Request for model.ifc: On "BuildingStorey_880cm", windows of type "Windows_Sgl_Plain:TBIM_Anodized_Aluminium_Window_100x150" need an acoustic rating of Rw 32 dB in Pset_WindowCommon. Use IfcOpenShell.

First a look at what the model holds.

```python
import ifcopenshell
import ifcopenshell.util.element

model = ifcopenshell.open("model.ifc")
print(model.schema)
storey = next(s for s in model.by_type("IfcBuildingStorey") if s.Name == "BuildingStorey_880cm")
windows = [e for e in ifcopenshell.util.element.get_decomposition(storey) if e.is_a("IfcWindow")]
seen = {}
for e in windows:
    element_type = ifcopenshell.util.element.get_type(e)
    key = (element_type.Name if element_type != e and element_type else None, ifcopenshell.util.element.get_pset(e, "Pset_WindowCommon", "AcousticRating"))
    seen[key] = seen.get(key, 0) + 1
for (name, value), count in sorted(seen.items(), key=str):
    print(count, "x", name, "|", value)
```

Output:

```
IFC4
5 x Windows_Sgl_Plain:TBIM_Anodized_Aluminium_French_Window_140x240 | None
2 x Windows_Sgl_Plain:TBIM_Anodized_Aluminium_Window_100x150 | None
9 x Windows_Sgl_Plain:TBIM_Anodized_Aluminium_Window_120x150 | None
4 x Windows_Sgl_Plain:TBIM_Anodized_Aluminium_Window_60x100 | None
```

```python
import ifcopenshell
import ifcopenshell.api.pset
import ifcopenshell.util.element

model = ifcopenshell.open("model.ifc")

storey = next(s for s in model.by_type("IfcBuildingStorey") if s.Name == "BuildingStorey_880cm")
windows = [e for e in ifcopenshell.util.element.get_decomposition(storey) if e.is_a("IfcWindow")]

count = 0
for e in windows:
    element_type = ifcopenshell.util.element.get_type(e)
    if element_type in (None, e) or element_type.Name != "Windows_Sgl_Plain:TBIM_Anodized_Aluminium_Window_100x150":
        continue
    # add_pset returns the element's existing set when there is one.
    pset = ifcopenshell.api.pset.add_pset(model, product=e, name="Pset_WindowCommon")
    ifcopenshell.api.pset.edit_pset(model, pset=pset, properties={"AcousticRating": "Rw 32 dB"})
    count += 1

print(count, "windows updated")

model.write("model_edited.ifc")
```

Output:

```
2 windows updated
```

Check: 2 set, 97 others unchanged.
